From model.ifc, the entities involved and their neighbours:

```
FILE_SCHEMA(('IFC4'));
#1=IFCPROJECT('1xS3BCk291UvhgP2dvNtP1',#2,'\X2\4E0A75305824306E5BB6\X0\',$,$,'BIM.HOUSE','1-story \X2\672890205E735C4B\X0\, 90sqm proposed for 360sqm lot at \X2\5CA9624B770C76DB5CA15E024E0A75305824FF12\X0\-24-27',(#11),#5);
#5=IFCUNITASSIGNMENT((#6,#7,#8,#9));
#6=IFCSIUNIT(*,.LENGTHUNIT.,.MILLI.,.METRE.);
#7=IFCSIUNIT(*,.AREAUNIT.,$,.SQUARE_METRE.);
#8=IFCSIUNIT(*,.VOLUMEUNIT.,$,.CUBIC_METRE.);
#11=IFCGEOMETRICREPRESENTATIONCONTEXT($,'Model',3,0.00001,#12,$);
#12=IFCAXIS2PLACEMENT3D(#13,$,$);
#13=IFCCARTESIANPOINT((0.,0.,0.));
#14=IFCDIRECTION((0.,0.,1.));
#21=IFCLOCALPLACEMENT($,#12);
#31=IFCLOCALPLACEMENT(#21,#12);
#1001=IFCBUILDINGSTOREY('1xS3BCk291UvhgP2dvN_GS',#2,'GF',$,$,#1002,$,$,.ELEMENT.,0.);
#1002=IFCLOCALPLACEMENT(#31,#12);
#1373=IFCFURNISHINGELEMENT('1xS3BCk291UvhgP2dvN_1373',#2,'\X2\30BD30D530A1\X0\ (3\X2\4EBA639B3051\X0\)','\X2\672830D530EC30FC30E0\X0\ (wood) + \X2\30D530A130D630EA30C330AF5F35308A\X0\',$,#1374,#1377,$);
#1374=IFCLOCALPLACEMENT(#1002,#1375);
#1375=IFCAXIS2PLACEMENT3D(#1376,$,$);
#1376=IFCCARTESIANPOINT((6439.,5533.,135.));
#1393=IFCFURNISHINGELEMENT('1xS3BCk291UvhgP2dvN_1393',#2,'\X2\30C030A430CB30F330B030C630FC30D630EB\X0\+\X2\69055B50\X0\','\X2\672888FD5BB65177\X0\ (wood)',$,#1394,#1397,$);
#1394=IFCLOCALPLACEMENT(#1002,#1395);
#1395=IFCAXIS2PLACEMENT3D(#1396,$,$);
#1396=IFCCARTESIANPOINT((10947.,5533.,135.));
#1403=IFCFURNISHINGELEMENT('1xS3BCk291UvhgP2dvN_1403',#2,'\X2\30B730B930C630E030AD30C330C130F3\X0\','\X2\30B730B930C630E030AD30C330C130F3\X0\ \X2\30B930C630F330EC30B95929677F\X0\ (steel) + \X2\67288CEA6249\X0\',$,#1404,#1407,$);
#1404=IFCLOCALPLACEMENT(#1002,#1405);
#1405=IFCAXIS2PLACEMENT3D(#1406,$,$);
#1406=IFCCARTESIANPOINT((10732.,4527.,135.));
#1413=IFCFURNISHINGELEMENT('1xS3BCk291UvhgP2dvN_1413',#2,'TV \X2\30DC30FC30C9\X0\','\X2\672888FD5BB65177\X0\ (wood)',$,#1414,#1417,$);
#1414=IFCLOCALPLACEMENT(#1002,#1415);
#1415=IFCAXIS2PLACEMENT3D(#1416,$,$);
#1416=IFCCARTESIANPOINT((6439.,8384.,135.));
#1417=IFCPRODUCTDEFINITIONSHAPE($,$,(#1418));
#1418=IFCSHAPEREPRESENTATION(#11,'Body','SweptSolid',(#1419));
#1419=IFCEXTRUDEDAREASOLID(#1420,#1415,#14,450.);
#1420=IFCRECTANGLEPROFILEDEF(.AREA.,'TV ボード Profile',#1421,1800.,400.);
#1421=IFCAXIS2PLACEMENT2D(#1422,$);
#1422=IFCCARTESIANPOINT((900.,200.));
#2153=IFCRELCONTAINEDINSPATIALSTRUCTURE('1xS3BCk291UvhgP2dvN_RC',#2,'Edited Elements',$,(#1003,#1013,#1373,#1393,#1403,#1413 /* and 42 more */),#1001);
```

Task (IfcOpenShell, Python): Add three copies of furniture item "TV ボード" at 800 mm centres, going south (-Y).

```python
import numpy as np
import ifcopenshell
import ifcopenshell.api.geometry
import ifcopenshell.api.root
import ifcopenshell.util.element
import ifcopenshell.util.placement

model = ifcopenshell.open("model.ifc")


def reuse_history(source, copy):
    """copy_class also copies each property set's owner history, people and application; keep the originals."""
    for rel in copy.IsDefinedBy:
        if rel.is_a("IfcRelDefinesByProperties") and (history := rel.RelatingPropertyDefinition.OwnerHistory):
            rel.RelatingPropertyDefinition.OwnerHistory = source.OwnerHistory
            ifcopenshell.util.element.remove_deep2(model, history)


source = model.by_guid("1xS3BCk291UvhgP2dvN_1413")
base = ifcopenshell.util.placement.get_local_placement(source.ObjectPlacement)
step = np.array([0.0, -1.0, 0.0]) * 800.0

for i in range(1, 4):
    copy = ifcopenshell.api.root.copy_class(model, product=source)
    copy.Representation = ifcopenshell.util.element.copy_deep(
        model, source.Representation, exclude=["IfcGeometricRepresentationContext", "IfcRepresentationMap"]
    )
    reuse_history(source, copy)
    matrix = base.copy()
    matrix[:3, 3] += i * step
    print("added at", matrix[:3, 3].round(3) + 0.0)
    ifcopenshell.api.geometry.edit_object_placement(model, product=copy, matrix=matrix, is_si=False)

model.write("model-out.ifc")
```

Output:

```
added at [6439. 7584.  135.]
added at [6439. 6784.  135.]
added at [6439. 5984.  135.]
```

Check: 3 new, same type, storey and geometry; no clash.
